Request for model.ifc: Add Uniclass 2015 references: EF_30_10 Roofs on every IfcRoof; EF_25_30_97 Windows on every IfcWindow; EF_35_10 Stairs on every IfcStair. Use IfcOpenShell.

First a look at what the model holds.

```python
import ifcopenshell

model = ifcopenshell.open("model.ifc")
print(model.schema)
print("classifications:", [c.Name for c in model.by_type("IfcClassification")])
for ifc_class in ("IfcDoor", "IfcRoof", "IfcStair", "IfcWall", "IfcWindow"):
    print(ifc_class, len(model.by_type(ifc_class)))
```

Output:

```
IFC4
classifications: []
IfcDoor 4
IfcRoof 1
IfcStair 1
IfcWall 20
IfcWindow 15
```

```python
import ifcopenshell
import ifcopenshell.api.classification

model = ifcopenshell.open("model.ifc")

system = ifcopenshell.api.classification.add_classification(model, classification="Uniclass 2015")

codes = {
    "IfcRoof": ("EF_30_10", "Roofs"),
    "IfcWindow": ("EF_25_30_97", "Windows"),
    "IfcStair": ("EF_35_10", "Stairs"),
}
for ifc_class, (code, name) in codes.items():
    products = model.by_type(ifc_class)
    ifcopenshell.api.classification.add_reference(
        model, products=products, classification=system, identification=code, name=name
    )
    print(code, len(products))

model.write("model-out.ifc")
```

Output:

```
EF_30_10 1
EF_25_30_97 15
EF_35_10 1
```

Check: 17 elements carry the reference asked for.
